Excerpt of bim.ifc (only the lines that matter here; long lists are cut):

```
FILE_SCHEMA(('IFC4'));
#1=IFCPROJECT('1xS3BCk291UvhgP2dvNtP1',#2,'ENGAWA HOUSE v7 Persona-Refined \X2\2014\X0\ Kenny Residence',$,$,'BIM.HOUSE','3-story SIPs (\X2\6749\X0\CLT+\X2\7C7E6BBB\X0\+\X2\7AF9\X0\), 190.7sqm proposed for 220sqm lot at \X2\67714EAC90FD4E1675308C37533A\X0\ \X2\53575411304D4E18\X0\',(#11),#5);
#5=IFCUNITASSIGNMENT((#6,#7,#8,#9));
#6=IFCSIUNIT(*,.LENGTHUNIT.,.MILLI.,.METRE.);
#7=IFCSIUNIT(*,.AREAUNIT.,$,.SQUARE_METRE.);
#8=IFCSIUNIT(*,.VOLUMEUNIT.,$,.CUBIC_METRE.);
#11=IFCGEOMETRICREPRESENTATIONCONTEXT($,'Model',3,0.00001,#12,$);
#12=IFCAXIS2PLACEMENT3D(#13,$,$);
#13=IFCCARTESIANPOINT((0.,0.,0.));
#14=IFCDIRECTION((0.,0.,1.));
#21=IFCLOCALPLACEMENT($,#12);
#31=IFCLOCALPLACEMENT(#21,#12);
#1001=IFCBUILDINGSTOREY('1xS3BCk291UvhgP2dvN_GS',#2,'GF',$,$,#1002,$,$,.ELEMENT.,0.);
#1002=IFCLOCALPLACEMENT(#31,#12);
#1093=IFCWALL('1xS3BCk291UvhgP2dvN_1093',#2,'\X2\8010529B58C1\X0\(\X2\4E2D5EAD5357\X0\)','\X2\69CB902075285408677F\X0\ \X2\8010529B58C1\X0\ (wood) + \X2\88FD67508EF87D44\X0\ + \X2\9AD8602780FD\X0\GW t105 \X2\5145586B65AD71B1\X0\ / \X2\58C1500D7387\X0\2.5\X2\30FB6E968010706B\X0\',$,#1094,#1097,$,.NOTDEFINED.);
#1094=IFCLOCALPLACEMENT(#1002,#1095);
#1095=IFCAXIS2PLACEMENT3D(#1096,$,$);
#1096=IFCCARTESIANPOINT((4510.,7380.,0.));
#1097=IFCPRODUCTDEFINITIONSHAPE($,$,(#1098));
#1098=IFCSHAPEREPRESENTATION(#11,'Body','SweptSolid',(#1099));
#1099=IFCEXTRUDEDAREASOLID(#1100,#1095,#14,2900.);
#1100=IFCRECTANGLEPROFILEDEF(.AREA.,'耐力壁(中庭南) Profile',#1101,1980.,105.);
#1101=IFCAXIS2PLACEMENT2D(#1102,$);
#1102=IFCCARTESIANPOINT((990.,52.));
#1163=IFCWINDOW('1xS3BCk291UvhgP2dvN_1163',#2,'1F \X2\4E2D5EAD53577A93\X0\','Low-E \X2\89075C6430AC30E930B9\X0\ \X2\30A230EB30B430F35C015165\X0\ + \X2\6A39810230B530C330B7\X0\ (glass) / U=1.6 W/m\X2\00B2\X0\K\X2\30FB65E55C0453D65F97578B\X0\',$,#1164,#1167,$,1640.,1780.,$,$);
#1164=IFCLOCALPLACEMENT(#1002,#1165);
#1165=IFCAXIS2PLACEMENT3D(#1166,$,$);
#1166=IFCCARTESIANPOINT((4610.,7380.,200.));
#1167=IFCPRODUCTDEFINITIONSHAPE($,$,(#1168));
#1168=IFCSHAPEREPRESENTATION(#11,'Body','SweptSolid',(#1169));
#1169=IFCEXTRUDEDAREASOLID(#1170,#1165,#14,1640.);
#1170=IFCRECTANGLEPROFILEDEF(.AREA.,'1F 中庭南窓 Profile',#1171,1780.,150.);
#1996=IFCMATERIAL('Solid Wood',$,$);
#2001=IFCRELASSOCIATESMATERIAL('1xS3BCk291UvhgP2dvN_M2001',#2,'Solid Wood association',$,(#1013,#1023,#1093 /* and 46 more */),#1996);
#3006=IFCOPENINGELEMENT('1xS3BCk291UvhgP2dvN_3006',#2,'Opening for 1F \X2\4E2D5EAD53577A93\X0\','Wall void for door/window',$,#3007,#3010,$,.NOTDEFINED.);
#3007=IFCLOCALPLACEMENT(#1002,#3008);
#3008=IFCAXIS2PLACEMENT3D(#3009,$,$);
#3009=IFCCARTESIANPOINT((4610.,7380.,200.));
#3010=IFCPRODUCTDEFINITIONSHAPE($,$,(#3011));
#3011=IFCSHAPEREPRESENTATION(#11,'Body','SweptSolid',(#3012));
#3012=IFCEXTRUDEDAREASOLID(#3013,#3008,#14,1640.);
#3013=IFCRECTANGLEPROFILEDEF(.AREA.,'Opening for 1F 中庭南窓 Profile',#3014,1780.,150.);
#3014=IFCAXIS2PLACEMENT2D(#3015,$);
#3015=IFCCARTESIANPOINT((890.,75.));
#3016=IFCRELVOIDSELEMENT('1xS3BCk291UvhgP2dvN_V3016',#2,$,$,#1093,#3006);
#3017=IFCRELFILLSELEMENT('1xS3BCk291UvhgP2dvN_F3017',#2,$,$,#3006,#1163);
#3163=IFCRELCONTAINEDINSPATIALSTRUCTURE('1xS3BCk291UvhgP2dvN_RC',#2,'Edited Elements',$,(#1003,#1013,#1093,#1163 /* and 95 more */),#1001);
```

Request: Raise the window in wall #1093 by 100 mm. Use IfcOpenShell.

```python
import numpy as np
import ifcopenshell
import ifcopenshell.api.geometry
import ifcopenshell.util.placement
import ifcopenshell.util.unit

model = ifcopenshell.open("bim.ifc")
unit_scale = ifcopenshell.util.unit.calculate_unit_scale(model)

window = model.by_guid("1xS3BCk291UvhgP2dvN_1163")
opening = window.FillsVoids[0].RelatingOpeningElement
dz = 0.1 / unit_scale

shift = np.array([0.0, 0.0, dz])
# The window is not placed relative to its opening, so move both.
for product in (opening, window):
    matrix = ifcopenshell.util.placement.get_local_placement(product.ObjectPlacement)
    matrix[:3, 3] += shift
    ifcopenshell.api.geometry.edit_object_placement(model, product=product, matrix=matrix, is_si=False)

print(f"moved by {dz * unit_scale:+.3f} m")

model.write("bim_updated.ifc")
```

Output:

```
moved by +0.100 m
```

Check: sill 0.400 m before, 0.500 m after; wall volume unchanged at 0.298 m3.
